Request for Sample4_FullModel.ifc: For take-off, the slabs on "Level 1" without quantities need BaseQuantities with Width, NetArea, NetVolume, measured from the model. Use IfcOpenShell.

First a look at what the model holds.

```python
import ifcopenshell
import ifcopenshell.util.element
import ifcopenshell.util.unit

model = ifcopenshell.open("Sample4_FullModel.ifc")
print(model.schema)
for unit_type in ("LENGTHUNIT", "AREAUNIT", "VOLUMEUNIT"):
    print(unit_type, ifcopenshell.util.unit.calculate_unit_scale(model, unit_type))
storey = next(s for s in model.by_type("IfcBuildingStorey") if s.Name == "Level 1")
slabs = [e for e in ifcopenshell.util.element.get_decomposition(storey) if e.is_a("IfcSlab")]
for e in sorted(slabs, key=lambda e: e.id()):
    print(e.id(), e.is_a(), e.Name, list(ifcopenshell.util.element.get_psets(e, qtos_only=True)), sep=" | ")
```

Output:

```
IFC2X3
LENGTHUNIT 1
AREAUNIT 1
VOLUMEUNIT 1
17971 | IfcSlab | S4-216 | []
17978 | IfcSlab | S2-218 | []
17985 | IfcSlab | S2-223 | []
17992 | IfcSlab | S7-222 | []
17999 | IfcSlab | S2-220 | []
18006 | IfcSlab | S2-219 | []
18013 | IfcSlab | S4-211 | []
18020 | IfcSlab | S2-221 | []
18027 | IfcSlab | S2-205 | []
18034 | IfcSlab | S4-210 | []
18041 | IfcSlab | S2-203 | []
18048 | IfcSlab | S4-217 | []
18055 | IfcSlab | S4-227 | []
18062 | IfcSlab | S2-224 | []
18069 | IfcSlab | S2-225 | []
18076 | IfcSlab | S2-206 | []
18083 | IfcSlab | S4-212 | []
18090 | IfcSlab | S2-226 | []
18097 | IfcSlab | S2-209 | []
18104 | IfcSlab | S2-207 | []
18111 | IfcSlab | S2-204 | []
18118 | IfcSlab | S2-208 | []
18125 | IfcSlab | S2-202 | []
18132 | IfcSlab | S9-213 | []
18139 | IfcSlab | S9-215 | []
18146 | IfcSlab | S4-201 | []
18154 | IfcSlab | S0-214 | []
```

```python
import ifcopenshell
import ifcopenshell.api.pset
import ifcopenshell.geom
import ifcopenshell.util.element
import ifcopenshell.util.shape
import ifcopenshell.util.unit

model = ifcopenshell.open("Sample4_FullModel.ifc")
unit_scale = ifcopenshell.util.unit.calculate_unit_scale(model)
area_scale = ifcopenshell.util.unit.calculate_unit_scale(model, "AREAUNIT")
volume_scale = ifcopenshell.util.unit.calculate_unit_scale(model, "VOLUMEUNIT")
settings = ifcopenshell.geom.settings()

storey = next(s for s in model.by_type("IfcBuildingStorey") if s.Name == "Level 1")
slabs = [e for e in ifcopenshell.util.element.get_decomposition(storey) if e.is_a("IfcSlab")]

for e in sorted(slabs, key=lambda e: e.id()):
    if ifcopenshell.util.element.get_psets(e, qtos_only=True, should_inherit=False):
        continue
    # Geometry comes back in metres, in the element's own axes.
    shape = ifcopenshell.geom.create_shape(settings, e)
    values = {
        "Width": ifcopenshell.util.shape.get_z(shape.geometry) / unit_scale,
        "NetArea": ifcopenshell.util.shape.get_footprint_area(shape.geometry) / area_scale,
        "NetVolume": ifcopenshell.util.shape.get_volume(shape.geometry) / volume_scale,
    }
    qto = ifcopenshell.api.pset.add_qto(model, product=e, name="BaseQuantities")
    ifcopenshell.api.pset.edit_qto(model, qto=qto, properties=values)
    print(e.id(), {k: round(v, 3) for k, v in values.items()})

model.write("Sample4_FullModel_updated.ifc")
```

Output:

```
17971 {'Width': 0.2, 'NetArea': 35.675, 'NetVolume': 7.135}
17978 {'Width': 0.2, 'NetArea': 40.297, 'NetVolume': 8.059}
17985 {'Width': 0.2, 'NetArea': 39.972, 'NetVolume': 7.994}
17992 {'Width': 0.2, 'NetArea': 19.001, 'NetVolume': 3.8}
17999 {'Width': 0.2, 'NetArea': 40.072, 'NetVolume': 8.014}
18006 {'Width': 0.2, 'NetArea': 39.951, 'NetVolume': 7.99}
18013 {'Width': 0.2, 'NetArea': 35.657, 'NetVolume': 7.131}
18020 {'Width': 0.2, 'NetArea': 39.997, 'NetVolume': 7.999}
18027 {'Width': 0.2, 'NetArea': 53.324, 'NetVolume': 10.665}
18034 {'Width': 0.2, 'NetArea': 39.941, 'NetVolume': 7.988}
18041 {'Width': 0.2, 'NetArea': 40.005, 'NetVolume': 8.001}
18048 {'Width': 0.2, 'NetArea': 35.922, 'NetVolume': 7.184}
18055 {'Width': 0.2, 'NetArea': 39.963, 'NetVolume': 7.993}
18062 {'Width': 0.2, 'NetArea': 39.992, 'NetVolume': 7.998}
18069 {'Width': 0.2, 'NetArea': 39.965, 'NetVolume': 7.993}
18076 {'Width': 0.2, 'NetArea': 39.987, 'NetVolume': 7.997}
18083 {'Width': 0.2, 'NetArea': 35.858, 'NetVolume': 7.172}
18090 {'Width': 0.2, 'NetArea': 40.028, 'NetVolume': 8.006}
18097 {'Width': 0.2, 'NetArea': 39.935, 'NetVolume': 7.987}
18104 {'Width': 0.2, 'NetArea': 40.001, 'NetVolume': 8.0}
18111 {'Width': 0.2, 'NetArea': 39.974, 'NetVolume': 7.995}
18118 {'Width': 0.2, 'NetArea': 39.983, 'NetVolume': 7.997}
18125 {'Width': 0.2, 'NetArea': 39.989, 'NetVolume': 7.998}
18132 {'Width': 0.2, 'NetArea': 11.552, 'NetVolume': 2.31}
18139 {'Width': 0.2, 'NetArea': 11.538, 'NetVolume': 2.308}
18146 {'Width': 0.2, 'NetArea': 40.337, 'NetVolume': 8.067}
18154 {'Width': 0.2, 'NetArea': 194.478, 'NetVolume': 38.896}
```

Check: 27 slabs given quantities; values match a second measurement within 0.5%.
